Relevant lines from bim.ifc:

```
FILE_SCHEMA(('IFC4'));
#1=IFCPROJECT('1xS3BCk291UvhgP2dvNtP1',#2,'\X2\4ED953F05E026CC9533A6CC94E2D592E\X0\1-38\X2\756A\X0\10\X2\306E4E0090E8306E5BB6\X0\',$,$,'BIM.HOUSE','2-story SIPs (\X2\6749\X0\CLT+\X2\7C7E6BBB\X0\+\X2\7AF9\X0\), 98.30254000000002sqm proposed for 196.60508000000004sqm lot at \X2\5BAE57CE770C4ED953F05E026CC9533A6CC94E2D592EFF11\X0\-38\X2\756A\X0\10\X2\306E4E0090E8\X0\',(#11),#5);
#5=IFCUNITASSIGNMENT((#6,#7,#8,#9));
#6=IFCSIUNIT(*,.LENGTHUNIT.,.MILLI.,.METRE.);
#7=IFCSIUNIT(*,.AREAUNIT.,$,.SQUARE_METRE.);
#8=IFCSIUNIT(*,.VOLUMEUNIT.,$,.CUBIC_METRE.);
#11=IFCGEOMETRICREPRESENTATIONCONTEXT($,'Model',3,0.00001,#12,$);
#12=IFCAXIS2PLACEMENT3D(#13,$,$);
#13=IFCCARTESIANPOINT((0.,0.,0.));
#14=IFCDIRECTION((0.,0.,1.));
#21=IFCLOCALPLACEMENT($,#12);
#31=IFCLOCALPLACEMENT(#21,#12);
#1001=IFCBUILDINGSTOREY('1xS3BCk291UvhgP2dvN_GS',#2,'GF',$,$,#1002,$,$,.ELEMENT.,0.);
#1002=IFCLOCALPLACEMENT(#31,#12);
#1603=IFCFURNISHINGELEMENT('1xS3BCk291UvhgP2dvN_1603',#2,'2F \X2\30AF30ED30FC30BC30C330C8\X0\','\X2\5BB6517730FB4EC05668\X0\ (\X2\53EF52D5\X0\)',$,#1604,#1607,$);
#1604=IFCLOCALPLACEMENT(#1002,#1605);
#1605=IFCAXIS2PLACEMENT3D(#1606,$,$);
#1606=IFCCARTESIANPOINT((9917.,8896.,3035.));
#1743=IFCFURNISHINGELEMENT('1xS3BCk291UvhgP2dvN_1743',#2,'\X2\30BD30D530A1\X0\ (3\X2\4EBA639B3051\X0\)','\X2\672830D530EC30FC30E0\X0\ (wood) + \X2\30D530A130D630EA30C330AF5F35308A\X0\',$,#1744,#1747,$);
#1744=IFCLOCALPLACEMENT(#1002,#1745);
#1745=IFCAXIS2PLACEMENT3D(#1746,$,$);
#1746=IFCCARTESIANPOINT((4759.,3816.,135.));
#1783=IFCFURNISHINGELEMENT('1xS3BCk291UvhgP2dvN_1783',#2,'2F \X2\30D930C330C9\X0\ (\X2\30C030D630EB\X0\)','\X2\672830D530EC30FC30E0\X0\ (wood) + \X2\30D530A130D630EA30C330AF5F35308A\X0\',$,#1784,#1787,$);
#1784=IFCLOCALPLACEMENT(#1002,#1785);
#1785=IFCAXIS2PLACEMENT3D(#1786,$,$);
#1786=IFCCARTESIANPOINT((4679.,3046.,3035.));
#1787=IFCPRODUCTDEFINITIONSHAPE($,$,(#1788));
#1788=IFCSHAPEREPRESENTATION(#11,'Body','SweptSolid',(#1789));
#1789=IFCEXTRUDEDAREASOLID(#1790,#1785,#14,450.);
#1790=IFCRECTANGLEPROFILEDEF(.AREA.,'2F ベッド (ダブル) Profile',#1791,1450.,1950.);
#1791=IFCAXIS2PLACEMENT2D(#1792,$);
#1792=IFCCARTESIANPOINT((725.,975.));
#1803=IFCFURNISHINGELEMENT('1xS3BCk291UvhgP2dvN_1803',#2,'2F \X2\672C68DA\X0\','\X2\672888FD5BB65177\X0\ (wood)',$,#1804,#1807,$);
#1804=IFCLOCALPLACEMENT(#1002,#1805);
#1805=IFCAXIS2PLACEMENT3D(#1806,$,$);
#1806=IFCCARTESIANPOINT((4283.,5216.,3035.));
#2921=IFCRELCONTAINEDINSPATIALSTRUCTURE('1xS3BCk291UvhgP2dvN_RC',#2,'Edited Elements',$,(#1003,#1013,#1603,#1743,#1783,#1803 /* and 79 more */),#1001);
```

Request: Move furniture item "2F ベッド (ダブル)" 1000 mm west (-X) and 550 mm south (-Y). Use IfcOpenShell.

```python
import ifcopenshell
import ifcopenshell.api.geometry
import ifcopenshell.util.placement
import ifcopenshell.util.unit

model = ifcopenshell.open("bim.ifc")
unit_scale = ifcopenshell.util.unit.calculate_unit_scale(model)

item = model.by_guid("1xS3BCk291UvhgP2dvN_1783")
matrix = ifcopenshell.util.placement.get_local_placement(item.ObjectPlacement)
matrix[0, 3] -= 1 / unit_scale
matrix[1, 3] -= 0.55 / unit_scale
ifcopenshell.api.geometry.edit_object_placement(model, product=item, matrix=matrix, is_si=False)

print(ifcopenshell.util.placement.get_local_placement(item.ObjectPlacement).round(3) + 0.0)

model.write("bim-out.ifc")
```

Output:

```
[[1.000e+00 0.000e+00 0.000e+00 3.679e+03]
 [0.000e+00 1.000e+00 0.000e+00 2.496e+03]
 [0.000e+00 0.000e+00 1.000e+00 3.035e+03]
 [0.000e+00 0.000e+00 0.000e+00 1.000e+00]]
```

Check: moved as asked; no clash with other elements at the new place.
